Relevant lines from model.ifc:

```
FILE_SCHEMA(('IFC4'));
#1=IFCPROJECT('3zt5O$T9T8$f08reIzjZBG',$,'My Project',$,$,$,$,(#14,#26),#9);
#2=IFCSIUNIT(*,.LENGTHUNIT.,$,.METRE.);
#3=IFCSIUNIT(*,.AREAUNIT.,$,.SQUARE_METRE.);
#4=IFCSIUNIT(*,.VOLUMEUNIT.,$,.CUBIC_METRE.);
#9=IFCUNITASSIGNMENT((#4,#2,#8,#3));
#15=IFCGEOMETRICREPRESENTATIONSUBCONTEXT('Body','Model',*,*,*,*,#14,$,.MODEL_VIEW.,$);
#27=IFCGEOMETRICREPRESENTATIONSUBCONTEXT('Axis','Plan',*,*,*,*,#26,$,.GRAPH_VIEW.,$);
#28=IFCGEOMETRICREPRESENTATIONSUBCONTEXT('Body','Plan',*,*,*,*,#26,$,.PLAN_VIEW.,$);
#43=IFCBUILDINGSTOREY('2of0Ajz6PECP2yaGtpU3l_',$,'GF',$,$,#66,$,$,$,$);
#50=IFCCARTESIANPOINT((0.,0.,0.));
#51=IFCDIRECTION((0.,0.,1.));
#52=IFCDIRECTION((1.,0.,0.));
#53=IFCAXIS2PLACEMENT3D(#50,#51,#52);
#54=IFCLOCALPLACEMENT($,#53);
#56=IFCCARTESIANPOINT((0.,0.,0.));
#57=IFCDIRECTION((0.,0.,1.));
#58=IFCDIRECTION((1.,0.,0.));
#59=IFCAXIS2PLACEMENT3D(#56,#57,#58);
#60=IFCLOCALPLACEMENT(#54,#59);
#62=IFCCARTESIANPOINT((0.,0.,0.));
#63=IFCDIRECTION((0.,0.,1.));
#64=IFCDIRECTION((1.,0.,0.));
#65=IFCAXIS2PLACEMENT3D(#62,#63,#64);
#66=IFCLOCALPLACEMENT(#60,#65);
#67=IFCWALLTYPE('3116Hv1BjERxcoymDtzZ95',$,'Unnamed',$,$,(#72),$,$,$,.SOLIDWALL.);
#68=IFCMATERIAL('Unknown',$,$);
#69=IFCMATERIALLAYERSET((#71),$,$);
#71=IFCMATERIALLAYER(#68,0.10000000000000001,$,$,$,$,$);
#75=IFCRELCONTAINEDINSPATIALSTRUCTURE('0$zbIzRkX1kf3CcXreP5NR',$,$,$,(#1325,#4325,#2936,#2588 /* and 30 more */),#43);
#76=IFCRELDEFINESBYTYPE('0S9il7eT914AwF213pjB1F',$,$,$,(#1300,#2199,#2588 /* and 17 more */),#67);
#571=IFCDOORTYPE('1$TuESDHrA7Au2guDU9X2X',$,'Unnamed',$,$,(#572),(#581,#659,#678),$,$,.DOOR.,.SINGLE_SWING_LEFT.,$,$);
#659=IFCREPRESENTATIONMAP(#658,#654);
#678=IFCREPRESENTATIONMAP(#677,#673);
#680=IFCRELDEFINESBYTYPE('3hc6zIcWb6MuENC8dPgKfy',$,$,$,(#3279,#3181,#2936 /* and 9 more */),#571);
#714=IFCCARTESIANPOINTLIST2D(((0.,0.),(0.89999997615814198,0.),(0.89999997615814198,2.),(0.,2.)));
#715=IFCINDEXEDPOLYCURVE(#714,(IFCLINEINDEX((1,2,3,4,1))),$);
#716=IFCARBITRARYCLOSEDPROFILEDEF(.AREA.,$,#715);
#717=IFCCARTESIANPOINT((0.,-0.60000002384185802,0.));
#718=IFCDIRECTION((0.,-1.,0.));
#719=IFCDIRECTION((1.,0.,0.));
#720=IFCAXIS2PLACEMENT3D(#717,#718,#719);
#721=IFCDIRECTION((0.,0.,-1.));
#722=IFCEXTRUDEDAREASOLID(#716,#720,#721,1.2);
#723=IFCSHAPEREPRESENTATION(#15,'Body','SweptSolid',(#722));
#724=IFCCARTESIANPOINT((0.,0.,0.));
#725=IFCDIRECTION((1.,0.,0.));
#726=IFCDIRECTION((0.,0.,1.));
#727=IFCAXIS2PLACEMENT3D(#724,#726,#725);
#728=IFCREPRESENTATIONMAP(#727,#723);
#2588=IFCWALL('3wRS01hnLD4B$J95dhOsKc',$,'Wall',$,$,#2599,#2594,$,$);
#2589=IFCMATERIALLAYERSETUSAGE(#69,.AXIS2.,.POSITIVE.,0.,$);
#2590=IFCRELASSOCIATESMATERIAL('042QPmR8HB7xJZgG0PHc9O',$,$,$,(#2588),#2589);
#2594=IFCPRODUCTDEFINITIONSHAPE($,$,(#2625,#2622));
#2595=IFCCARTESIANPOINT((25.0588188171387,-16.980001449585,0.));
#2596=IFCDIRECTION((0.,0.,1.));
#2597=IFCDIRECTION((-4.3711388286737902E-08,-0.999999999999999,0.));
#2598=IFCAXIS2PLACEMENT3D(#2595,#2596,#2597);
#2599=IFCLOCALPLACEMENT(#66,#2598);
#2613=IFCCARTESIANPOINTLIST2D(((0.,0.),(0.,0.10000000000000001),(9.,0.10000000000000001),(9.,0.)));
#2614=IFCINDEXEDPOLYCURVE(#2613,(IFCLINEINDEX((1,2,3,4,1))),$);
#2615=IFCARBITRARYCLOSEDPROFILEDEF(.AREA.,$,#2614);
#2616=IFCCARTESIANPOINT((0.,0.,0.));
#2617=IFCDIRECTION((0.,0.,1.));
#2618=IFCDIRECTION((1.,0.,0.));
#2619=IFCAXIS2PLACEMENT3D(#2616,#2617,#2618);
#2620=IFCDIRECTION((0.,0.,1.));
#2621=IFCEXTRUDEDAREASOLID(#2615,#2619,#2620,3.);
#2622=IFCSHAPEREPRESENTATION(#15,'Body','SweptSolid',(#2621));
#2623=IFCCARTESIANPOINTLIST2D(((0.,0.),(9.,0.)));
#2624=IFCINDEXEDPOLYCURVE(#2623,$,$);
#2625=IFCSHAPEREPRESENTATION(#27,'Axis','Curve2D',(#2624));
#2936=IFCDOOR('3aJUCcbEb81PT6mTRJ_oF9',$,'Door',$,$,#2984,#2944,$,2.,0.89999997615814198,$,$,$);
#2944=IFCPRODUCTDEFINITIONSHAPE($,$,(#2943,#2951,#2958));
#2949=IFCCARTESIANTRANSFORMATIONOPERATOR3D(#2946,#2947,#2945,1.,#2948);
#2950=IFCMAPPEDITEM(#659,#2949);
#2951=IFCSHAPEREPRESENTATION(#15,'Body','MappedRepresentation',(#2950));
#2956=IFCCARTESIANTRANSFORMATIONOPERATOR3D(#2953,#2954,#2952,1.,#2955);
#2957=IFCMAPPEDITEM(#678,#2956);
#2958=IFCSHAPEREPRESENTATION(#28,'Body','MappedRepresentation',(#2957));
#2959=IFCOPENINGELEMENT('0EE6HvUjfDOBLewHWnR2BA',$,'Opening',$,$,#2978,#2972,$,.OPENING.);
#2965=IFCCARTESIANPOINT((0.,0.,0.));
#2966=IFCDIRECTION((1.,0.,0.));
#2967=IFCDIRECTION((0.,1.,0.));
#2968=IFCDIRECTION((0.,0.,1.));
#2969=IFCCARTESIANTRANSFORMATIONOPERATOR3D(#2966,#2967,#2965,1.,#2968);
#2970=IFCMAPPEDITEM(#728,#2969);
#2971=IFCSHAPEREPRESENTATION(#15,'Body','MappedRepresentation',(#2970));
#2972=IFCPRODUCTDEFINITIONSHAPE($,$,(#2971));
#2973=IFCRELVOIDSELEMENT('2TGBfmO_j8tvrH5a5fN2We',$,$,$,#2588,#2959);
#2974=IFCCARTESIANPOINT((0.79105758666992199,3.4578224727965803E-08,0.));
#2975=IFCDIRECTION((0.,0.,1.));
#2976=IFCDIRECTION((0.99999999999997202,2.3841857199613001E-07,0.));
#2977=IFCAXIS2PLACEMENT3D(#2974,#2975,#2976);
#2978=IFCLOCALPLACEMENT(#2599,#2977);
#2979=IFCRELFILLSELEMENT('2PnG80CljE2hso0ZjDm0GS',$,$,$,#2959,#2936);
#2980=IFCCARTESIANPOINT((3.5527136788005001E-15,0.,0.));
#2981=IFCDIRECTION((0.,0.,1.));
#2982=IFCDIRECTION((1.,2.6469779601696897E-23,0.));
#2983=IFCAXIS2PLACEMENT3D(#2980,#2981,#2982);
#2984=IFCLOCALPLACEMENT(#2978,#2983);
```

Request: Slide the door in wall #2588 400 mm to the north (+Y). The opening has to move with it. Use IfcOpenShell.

```python
import ifcopenshell
import ifcopenshell.api.geometry
import ifcopenshell.util.placement
import ifcopenshell.util.unit

model = ifcopenshell.open("model.ifc")
unit_scale = ifcopenshell.util.unit.calculate_unit_scale(model)

door = model.by_guid("3aJUCcbEb81PT6mTRJ_oF9")
opening = door.FillsVoids[0].RelatingOpeningElement
wall = opening.VoidsElements[0].RelatingBuildingElement

wall_matrix = ifcopenshell.util.placement.get_local_placement(wall.ObjectPlacement)
shift = wall_matrix[:3, 0] * -0.4 / unit_scale
before = ifcopenshell.util.placement.get_local_placement(door.ObjectPlacement)[:3, 3].copy()

# The door is placed relative to its opening, so it follows when the opening moves.
matrix = ifcopenshell.util.placement.get_local_placement(opening.ObjectPlacement)
matrix[:3, 3] += shift
ifcopenshell.api.geometry.edit_object_placement(
    model, product=opening, matrix=matrix, is_si=False, should_transform_children=True
)

after = ifcopenshell.util.placement.get_local_placement(door.ObjectPlacement)[:3, 3]
print("door moved by", (after - before).round(3) + 0.0)

model.write("model_edited.ifc")
```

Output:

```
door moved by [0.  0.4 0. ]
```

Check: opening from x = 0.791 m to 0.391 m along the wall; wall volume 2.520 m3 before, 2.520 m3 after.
